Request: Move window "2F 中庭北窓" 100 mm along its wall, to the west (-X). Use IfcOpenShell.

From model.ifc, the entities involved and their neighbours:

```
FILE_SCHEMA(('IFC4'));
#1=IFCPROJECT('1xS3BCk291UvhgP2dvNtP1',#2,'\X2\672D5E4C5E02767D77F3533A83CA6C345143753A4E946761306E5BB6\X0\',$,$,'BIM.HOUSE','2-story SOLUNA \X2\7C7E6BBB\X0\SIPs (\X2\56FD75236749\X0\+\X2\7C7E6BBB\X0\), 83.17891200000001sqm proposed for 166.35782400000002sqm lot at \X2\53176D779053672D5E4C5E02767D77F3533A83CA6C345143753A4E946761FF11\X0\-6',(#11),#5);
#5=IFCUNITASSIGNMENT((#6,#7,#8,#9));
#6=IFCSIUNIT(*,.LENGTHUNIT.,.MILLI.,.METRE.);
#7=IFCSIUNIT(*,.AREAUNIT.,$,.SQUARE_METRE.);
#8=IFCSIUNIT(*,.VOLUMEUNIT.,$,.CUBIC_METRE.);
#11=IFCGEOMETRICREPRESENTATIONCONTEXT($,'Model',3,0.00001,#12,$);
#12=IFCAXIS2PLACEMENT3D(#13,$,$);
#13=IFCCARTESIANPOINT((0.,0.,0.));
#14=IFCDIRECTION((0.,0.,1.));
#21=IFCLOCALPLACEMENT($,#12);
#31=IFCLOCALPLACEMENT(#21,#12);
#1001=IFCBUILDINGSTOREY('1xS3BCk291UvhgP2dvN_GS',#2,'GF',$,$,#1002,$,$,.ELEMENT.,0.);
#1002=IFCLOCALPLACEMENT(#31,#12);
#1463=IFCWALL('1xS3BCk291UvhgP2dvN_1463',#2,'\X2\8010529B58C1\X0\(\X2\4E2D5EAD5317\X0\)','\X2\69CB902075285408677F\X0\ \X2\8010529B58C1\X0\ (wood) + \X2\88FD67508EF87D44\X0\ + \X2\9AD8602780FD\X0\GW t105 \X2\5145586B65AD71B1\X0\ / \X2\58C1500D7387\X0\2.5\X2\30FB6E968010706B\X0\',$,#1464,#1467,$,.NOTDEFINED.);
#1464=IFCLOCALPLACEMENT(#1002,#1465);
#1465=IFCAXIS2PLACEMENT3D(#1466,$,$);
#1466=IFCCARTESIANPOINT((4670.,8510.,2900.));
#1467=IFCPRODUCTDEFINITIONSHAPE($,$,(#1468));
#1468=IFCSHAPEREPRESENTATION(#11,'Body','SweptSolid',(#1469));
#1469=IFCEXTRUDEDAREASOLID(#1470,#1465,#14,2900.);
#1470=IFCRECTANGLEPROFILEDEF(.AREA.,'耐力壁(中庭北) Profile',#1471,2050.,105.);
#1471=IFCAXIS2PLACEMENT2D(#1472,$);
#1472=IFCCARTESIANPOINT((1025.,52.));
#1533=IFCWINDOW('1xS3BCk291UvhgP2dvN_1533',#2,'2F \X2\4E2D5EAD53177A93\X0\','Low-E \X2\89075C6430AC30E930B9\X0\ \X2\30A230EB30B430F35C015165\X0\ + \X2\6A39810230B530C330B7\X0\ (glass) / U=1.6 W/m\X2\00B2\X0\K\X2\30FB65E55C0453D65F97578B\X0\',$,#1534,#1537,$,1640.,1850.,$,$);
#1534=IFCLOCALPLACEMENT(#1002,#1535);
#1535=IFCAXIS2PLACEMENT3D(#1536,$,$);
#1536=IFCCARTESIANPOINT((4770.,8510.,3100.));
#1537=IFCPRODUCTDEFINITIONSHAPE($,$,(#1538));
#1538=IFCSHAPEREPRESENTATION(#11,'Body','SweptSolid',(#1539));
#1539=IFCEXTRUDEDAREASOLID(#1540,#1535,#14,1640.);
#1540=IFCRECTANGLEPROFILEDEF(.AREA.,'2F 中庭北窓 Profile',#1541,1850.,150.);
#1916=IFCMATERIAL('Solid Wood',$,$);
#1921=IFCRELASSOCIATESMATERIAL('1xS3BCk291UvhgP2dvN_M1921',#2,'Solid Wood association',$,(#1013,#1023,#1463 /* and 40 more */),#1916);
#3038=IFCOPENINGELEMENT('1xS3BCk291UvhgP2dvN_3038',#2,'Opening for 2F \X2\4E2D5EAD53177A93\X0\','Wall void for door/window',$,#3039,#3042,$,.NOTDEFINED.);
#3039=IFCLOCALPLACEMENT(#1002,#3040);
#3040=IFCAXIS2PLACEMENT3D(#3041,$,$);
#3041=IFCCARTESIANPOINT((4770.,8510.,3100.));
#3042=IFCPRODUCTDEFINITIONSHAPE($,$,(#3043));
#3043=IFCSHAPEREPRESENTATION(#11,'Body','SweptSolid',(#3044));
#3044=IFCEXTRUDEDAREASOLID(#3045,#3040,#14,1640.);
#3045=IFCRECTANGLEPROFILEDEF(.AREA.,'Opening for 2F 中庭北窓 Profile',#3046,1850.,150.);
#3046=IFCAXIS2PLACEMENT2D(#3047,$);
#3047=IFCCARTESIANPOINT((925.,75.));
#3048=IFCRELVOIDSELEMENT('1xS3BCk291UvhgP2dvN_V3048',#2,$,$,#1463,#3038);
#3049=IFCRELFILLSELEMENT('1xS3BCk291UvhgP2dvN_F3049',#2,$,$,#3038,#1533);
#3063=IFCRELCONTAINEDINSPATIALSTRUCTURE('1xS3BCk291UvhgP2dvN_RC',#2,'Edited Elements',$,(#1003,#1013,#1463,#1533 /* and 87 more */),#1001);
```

```python
import ifcopenshell
import ifcopenshell.api.geometry
import ifcopenshell.util.placement
import ifcopenshell.util.unit

model = ifcopenshell.open("model.ifc")
unit_scale = ifcopenshell.util.unit.calculate_unit_scale(model)

window = model.by_id(1533)
opening = window.FillsVoids[0].RelatingOpeningElement
wall = opening.VoidsElements[0].RelatingBuildingElement

wall_matrix = ifcopenshell.util.placement.get_local_placement(wall.ObjectPlacement)
shift = wall_matrix[:3, 0] * -0.1 / unit_scale
before = ifcopenshell.util.placement.get_local_placement(window.ObjectPlacement)[:3, 3].copy()

# The window is not placed relative to its opening, so move both.
for product in (opening, window):
    matrix = ifcopenshell.util.placement.get_local_placement(product.ObjectPlacement)
    matrix[:3, 3] += shift
    ifcopenshell.api.geometry.edit_object_placement(model, product=product, matrix=matrix, is_si=False)

after = ifcopenshell.util.placement.get_local_placement(window.ObjectPlacement)[:3, 3]
print("window moved by", (after - before).round(3) + 0.0)

model.write("model_v2.ifc")
```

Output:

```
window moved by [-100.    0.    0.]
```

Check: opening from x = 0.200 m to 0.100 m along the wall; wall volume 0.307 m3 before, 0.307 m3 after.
